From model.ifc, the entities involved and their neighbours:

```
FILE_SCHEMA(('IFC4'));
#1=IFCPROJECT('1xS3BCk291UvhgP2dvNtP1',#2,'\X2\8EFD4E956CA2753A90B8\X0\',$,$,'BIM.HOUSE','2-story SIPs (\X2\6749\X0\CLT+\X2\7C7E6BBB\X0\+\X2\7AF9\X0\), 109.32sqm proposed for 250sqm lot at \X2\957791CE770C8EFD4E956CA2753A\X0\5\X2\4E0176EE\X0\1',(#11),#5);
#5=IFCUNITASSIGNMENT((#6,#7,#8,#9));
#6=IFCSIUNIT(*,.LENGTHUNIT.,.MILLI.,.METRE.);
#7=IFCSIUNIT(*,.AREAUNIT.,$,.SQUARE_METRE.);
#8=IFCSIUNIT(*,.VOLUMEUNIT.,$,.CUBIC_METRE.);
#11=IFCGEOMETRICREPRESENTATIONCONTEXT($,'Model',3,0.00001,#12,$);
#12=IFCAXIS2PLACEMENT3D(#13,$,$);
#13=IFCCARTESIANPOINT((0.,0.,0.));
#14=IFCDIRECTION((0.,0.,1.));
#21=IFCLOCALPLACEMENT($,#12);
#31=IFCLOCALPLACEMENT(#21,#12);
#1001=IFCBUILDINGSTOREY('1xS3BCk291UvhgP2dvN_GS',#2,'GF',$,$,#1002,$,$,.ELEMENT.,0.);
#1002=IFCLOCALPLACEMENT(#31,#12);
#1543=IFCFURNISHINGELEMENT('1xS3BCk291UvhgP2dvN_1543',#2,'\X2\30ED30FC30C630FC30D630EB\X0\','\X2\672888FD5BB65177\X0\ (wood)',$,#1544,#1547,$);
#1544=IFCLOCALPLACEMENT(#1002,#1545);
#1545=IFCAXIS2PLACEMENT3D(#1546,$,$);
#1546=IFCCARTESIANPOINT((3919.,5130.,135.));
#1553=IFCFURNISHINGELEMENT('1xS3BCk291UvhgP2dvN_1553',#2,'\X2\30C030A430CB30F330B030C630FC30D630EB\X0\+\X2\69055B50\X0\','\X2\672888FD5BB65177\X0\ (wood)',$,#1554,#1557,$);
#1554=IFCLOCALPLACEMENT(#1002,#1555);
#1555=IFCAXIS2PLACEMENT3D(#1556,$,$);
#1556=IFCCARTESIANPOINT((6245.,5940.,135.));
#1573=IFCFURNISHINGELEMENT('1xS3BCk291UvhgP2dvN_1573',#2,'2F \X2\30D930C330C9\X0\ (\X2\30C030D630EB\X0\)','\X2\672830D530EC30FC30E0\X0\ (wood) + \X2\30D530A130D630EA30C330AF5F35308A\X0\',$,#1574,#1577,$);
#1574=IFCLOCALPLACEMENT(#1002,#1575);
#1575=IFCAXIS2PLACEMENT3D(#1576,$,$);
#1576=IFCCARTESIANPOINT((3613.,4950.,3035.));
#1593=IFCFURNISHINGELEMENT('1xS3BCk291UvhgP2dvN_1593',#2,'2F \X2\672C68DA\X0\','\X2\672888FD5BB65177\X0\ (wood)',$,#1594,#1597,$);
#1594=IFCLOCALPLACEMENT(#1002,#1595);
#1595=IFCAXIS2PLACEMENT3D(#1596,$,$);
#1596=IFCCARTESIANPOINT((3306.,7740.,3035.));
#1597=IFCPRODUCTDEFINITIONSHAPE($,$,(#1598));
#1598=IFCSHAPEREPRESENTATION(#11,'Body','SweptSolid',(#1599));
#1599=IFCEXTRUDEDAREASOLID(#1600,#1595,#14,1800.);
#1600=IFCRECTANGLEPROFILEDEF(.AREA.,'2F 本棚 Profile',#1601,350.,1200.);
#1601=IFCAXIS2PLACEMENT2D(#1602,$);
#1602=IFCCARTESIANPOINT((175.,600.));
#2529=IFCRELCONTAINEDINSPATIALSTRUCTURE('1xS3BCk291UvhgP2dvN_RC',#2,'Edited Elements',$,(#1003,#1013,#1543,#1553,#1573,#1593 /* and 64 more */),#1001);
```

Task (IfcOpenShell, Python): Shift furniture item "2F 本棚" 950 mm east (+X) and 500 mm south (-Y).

```python
import ifcopenshell
import ifcopenshell.api.geometry
import ifcopenshell.util.placement
import ifcopenshell.util.unit

model = ifcopenshell.open("model.ifc")
unit_scale = ifcopenshell.util.unit.calculate_unit_scale(model)

item = model.by_guid("1xS3BCk291UvhgP2dvN_1593")
matrix = ifcopenshell.util.placement.get_local_placement(item.ObjectPlacement)
matrix[0, 3] += 0.95 / unit_scale
matrix[1, 3] -= 0.5 / unit_scale
ifcopenshell.api.geometry.edit_object_placement(model, product=item, matrix=matrix, is_si=False)

print(ifcopenshell.util.placement.get_local_placement(item.ObjectPlacement).round(3) + 0.0)

model.write("model_updated.ifc")
```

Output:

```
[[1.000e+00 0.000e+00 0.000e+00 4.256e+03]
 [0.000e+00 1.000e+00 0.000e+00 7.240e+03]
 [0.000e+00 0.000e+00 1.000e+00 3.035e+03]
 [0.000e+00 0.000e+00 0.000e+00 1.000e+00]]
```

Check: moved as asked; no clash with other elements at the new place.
